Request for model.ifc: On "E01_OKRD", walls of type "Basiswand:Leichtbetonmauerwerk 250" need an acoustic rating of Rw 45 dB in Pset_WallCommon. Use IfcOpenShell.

First a look at what the model holds.

```python
import ifcopenshell
import ifcopenshell.util.element

model = ifcopenshell.open("model.ifc")
print(model.schema)
storey = next(s for s in model.by_type("IfcBuildingStorey") if s.Name == "E01_OKRD")
walls = [e for e in ifcopenshell.util.element.get_decomposition(storey) if e.is_a("IfcWall")]
seen = {}
for e in walls:
    element_type = ifcopenshell.util.element.get_type(e)
    key = (element_type.Name if element_type != e and element_type else None, ifcopenshell.util.element.get_pset(e, "Pset_WallCommon", "AcousticRating"))
    seen[key] = seen.get(key, 0) + 1
for (name, value), count in sorted(seen.items(), key=str):
    print(count, "x", name, "|", value)
```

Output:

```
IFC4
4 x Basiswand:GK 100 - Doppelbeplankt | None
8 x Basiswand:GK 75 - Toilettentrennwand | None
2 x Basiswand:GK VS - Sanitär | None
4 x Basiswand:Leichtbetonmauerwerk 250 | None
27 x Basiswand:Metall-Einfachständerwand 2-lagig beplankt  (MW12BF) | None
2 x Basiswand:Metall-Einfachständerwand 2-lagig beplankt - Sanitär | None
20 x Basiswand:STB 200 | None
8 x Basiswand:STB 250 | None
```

```python
import ifcopenshell
import ifcopenshell.api.pset
import ifcopenshell.util.element

model = ifcopenshell.open("model.ifc")

storey = next(s for s in model.by_type("IfcBuildingStorey") if s.Name == "E01_OKRD")
walls = [e for e in ifcopenshell.util.element.get_decomposition(storey) if e.is_a("IfcWall")]

count = 0
for e in walls:
    element_type = ifcopenshell.util.element.get_type(e)
    if element_type in (None, e) or element_type.Name != "Basiswand:Leichtbetonmauerwerk 250":
        continue
    # add_pset returns the element's existing set when there is one.
    pset = ifcopenshell.api.pset.add_pset(model, product=e, name="Pset_WallCommon")
    ifcopenshell.api.pset.edit_pset(model, pset=pset, properties={"AcousticRating": "Rw 45 dB"})
    count += 1

print(count, "walls updated")

model.write("model-out.ifc")
```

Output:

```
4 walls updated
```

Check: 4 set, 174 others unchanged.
